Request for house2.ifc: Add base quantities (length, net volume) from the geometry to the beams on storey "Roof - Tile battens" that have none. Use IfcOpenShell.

First a look at what the model holds.

```python
import ifcopenshell
import ifcopenshell.util.element
import ifcopenshell.util.unit

model = ifcopenshell.open("house2.ifc")
print(model.schema)
for unit_type in ("LENGTHUNIT", "AREAUNIT", "VOLUMEUNIT"):
    print(unit_type, ifcopenshell.util.unit.calculate_unit_scale(model, unit_type))
storey = next(s for s in model.by_type("IfcBuildingStorey") if s.Name == "Roof - Tile battens")
beams = [e for e in ifcopenshell.util.element.get_decomposition(storey) if e.is_a("IfcBeam")]
for e in sorted(beams, key=lambda e: e.id()):
    print(e.id(), e.is_a(), e.Name, list(ifcopenshell.util.element.get_psets(e, qtos_only=True)), sep=" | ")
```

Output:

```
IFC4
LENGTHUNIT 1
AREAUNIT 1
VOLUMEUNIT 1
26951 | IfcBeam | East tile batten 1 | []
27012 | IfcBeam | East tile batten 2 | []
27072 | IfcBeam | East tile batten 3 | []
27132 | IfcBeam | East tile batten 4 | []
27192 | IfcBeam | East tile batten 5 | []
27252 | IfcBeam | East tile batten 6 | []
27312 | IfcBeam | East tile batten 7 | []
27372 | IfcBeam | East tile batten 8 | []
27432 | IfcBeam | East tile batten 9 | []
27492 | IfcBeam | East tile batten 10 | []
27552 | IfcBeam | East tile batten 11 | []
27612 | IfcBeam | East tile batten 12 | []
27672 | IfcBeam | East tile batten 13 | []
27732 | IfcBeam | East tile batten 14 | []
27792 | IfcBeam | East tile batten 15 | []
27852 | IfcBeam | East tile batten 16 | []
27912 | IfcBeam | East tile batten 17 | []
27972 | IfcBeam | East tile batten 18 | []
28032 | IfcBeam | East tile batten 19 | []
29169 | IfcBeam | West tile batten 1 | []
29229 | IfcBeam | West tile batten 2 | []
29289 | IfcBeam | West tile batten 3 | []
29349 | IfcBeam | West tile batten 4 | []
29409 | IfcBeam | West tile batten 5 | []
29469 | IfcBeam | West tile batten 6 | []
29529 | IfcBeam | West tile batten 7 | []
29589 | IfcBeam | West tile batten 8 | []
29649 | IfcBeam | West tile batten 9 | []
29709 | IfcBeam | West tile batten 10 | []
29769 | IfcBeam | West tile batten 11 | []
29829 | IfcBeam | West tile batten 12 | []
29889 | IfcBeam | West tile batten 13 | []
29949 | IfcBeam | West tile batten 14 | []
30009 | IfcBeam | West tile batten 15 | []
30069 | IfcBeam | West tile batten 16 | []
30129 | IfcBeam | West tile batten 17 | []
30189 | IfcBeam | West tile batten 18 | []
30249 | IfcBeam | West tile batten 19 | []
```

```python
import ifcopenshell
import ifcopenshell.api.pset
import ifcopenshell.geom
import ifcopenshell.util.element
import ifcopenshell.util.shape
import ifcopenshell.util.unit

model = ifcopenshell.open("house2.ifc")
unit_scale = ifcopenshell.util.unit.calculate_unit_scale(model)
volume_scale = ifcopenshell.util.unit.calculate_unit_scale(model, "VOLUMEUNIT")
settings = ifcopenshell.geom.settings()

storey = next(s for s in model.by_type("IfcBuildingStorey") if s.Name == "Roof - Tile battens")
beams = [e for e in ifcopenshell.util.element.get_decomposition(storey) if e.is_a("IfcBeam")]

for e in sorted(beams, key=lambda e: e.id()):
    if ifcopenshell.util.element.get_psets(e, qtos_only=True, should_inherit=False):
        continue
    # Geometry comes back in metres, in the element's own axes.
    shape = ifcopenshell.geom.create_shape(settings, e)
    values = {
        "Length": ifcopenshell.util.shape.get_max_xyz(shape.geometry) / unit_scale,
        "NetVolume": ifcopenshell.util.shape.get_volume(shape.geometry) / volume_scale,
    }
    qto = ifcopenshell.api.pset.add_qto(model, product=e, name="Qto_BeamBaseQuantities")
    ifcopenshell.api.pset.edit_qto(model, qto=qto, properties=values)
    print(e.id(), {k: round(v, 3) for k, v in values.items()})

model.write("house2_edited.ifc")
```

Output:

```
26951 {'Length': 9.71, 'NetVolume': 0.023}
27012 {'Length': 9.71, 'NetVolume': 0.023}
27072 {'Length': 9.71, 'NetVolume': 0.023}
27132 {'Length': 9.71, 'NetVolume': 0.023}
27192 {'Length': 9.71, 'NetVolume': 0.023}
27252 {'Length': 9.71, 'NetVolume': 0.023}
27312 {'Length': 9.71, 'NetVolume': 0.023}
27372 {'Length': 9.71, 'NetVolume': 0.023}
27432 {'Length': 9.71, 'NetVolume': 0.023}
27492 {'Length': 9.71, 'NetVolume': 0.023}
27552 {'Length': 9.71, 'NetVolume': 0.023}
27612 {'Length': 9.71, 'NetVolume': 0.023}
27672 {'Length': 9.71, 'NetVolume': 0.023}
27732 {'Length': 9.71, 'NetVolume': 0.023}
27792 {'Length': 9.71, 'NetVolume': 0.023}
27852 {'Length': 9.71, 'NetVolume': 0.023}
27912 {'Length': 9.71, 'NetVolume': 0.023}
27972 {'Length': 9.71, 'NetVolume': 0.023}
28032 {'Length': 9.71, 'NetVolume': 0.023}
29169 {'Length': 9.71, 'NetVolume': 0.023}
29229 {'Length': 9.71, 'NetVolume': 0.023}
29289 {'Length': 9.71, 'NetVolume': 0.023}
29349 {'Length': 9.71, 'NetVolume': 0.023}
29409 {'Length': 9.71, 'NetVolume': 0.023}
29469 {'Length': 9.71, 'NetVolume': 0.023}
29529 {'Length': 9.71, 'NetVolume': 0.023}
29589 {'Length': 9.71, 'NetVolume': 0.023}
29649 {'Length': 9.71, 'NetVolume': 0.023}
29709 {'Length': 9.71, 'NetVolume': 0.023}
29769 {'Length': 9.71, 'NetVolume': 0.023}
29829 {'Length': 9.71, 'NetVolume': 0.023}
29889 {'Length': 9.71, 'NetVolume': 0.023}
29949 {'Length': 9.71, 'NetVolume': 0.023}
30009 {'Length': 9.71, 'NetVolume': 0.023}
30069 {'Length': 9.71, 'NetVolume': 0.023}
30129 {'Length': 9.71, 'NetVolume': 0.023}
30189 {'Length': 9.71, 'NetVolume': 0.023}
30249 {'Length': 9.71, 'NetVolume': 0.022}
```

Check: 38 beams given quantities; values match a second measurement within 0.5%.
